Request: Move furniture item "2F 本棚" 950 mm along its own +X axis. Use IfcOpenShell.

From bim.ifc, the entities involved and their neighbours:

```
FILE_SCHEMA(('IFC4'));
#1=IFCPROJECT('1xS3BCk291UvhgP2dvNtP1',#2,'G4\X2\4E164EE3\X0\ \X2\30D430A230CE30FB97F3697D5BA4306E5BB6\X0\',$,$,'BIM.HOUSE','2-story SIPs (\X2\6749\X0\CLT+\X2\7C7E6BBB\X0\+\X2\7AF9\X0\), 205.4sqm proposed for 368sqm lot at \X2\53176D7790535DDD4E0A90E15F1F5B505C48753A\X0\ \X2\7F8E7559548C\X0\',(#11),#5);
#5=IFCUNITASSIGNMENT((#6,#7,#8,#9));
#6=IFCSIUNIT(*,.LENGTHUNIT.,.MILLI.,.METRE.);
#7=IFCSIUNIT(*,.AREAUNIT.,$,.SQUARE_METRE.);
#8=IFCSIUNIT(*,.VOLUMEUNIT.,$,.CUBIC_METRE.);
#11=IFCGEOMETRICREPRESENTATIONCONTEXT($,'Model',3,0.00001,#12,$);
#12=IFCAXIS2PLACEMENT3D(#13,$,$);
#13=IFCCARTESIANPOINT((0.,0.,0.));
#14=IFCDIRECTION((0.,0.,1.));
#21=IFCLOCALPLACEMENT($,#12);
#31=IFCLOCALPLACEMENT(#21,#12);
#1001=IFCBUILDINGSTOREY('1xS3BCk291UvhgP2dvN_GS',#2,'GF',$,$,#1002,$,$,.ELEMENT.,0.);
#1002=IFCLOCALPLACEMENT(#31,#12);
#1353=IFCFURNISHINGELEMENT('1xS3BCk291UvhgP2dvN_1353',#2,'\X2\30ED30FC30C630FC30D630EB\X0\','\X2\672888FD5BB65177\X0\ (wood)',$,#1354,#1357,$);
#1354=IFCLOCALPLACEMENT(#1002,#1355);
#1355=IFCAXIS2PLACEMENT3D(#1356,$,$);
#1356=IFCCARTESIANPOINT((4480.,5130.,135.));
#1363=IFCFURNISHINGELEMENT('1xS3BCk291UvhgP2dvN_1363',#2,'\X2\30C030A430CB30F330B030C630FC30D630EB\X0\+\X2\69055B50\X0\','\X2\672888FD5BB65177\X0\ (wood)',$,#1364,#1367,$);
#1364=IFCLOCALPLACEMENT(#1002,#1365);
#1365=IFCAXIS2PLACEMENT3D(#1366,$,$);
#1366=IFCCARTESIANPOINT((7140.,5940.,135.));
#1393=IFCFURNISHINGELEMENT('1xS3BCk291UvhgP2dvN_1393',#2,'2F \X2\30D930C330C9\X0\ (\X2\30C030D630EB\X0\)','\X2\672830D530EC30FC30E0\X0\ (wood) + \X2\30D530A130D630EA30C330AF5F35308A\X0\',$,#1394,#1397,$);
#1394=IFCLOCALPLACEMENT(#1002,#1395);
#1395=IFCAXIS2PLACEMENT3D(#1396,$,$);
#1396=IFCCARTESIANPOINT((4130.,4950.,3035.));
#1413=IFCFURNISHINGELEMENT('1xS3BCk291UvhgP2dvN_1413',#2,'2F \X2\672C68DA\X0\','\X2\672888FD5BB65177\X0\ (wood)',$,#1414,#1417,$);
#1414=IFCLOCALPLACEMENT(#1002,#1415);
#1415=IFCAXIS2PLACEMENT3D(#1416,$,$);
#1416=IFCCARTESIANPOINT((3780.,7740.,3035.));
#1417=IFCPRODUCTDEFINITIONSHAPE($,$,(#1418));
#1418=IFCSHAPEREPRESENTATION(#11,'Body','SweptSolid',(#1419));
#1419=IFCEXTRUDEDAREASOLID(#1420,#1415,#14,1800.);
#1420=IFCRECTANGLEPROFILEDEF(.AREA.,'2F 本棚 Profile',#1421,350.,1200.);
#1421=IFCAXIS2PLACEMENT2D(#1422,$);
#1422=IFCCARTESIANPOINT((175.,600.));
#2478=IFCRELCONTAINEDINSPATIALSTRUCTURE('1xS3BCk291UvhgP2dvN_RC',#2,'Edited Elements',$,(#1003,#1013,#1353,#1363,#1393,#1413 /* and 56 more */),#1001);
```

```python
import ifcopenshell
import ifcopenshell.api.geometry
import ifcopenshell.util.placement
import ifcopenshell.util.unit

model = ifcopenshell.open("bim.ifc")
unit_scale = ifcopenshell.util.unit.calculate_unit_scale(model)

item = model.by_guid("1xS3BCk291UvhgP2dvN_1413")
matrix = ifcopenshell.util.placement.get_local_placement(item.ObjectPlacement)
matrix[:3, 3] += matrix[:3, 0] * 0.95 / unit_scale
ifcopenshell.api.geometry.edit_object_placement(model, product=item, matrix=matrix, is_si=False)

print(ifcopenshell.util.placement.get_local_placement(item.ObjectPlacement).round(3) + 0.0)

model.write("bim_updated.ifc")
```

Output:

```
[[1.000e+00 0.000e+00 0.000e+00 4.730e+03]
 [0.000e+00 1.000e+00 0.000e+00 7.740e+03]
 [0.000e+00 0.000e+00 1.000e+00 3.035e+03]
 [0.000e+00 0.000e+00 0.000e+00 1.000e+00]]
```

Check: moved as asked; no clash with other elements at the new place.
